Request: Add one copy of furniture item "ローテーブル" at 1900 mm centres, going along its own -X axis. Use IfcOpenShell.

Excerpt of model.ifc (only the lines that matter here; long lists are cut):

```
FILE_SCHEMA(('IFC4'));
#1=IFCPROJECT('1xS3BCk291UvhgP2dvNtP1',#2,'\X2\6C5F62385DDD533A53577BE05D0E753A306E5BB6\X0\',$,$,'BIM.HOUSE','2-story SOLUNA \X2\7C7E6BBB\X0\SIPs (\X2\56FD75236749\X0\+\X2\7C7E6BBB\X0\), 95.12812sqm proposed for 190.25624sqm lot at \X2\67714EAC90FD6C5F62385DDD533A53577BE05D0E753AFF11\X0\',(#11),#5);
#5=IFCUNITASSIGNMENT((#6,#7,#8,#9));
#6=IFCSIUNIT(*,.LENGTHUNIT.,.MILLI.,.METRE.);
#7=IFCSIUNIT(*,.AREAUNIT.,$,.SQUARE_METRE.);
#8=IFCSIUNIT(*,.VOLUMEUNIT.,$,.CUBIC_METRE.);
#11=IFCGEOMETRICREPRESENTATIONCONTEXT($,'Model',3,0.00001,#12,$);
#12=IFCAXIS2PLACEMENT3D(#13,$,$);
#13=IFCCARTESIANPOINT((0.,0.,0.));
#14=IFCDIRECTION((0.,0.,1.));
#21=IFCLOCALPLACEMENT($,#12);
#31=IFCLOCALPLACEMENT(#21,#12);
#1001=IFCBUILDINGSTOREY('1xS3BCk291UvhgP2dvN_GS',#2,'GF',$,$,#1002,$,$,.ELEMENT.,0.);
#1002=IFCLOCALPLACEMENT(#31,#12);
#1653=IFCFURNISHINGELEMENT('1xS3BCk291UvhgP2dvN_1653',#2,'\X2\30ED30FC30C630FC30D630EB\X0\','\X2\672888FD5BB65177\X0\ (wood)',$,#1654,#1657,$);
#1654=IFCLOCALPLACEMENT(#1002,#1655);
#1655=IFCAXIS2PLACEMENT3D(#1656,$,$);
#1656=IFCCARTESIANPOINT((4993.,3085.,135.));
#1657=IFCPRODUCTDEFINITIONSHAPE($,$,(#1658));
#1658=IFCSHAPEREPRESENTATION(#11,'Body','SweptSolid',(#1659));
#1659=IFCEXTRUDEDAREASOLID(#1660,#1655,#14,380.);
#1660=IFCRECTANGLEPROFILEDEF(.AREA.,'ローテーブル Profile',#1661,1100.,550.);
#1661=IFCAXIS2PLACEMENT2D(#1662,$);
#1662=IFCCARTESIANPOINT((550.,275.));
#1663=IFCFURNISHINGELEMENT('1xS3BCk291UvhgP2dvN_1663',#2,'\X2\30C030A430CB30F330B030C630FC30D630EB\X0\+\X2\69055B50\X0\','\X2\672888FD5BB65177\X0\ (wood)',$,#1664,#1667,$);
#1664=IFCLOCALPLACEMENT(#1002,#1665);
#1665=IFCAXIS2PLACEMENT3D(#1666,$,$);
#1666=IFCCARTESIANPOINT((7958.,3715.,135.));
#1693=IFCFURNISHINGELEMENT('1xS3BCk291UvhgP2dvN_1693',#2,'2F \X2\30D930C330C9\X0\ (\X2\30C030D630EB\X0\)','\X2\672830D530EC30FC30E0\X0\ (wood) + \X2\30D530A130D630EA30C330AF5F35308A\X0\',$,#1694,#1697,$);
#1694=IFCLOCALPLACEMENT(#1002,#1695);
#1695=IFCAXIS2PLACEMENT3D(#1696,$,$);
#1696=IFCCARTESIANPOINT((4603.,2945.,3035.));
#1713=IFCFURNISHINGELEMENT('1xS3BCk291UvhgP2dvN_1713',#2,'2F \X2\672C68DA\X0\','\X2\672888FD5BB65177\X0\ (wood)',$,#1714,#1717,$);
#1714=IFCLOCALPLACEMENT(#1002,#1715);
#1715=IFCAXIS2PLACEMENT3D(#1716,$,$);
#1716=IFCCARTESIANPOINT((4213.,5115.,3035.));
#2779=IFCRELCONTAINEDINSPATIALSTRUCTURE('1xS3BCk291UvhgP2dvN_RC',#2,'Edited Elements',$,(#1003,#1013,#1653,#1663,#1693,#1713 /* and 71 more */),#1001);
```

```python
import ifcopenshell
import ifcopenshell.api.geometry
import ifcopenshell.api.root
import ifcopenshell.util.element
import ifcopenshell.util.placement
import ifcopenshell.util.unit

model = ifcopenshell.open("model.ifc")
unit_scale = ifcopenshell.util.unit.calculate_unit_scale(model)


def reuse_history(source, copy):
    """copy_class also copies each property set's owner history, people and application; keep the originals."""
    for rel in copy.IsDefinedBy:
        if rel.is_a("IfcRelDefinesByProperties") and (history := rel.RelatingPropertyDefinition.OwnerHistory):
            rel.RelatingPropertyDefinition.OwnerHistory = source.OwnerHistory
            ifcopenshell.util.element.remove_deep2(model, history)


source = model.by_guid("1xS3BCk291UvhgP2dvN_1653")
base = ifcopenshell.util.placement.get_local_placement(source.ObjectPlacement)
step = -base[:3, 0] * 1.9 / unit_scale

for i in range(1, 2):
    copy = ifcopenshell.api.root.copy_class(model, product=source)
    copy.Representation = ifcopenshell.util.element.copy_deep(
        model, source.Representation, exclude=["IfcGeometricRepresentationContext", "IfcRepresentationMap"]
    )
    reuse_history(source, copy)
    matrix = base.copy()
    matrix[:3, 3] += i * step
    print("added at", matrix[:3, 3].round(3) + 0.0)
    ifcopenshell.api.geometry.edit_object_placement(model, product=copy, matrix=matrix, is_si=False)

model.write("model_v2.ifc")
```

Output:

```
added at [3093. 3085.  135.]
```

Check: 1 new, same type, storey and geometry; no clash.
